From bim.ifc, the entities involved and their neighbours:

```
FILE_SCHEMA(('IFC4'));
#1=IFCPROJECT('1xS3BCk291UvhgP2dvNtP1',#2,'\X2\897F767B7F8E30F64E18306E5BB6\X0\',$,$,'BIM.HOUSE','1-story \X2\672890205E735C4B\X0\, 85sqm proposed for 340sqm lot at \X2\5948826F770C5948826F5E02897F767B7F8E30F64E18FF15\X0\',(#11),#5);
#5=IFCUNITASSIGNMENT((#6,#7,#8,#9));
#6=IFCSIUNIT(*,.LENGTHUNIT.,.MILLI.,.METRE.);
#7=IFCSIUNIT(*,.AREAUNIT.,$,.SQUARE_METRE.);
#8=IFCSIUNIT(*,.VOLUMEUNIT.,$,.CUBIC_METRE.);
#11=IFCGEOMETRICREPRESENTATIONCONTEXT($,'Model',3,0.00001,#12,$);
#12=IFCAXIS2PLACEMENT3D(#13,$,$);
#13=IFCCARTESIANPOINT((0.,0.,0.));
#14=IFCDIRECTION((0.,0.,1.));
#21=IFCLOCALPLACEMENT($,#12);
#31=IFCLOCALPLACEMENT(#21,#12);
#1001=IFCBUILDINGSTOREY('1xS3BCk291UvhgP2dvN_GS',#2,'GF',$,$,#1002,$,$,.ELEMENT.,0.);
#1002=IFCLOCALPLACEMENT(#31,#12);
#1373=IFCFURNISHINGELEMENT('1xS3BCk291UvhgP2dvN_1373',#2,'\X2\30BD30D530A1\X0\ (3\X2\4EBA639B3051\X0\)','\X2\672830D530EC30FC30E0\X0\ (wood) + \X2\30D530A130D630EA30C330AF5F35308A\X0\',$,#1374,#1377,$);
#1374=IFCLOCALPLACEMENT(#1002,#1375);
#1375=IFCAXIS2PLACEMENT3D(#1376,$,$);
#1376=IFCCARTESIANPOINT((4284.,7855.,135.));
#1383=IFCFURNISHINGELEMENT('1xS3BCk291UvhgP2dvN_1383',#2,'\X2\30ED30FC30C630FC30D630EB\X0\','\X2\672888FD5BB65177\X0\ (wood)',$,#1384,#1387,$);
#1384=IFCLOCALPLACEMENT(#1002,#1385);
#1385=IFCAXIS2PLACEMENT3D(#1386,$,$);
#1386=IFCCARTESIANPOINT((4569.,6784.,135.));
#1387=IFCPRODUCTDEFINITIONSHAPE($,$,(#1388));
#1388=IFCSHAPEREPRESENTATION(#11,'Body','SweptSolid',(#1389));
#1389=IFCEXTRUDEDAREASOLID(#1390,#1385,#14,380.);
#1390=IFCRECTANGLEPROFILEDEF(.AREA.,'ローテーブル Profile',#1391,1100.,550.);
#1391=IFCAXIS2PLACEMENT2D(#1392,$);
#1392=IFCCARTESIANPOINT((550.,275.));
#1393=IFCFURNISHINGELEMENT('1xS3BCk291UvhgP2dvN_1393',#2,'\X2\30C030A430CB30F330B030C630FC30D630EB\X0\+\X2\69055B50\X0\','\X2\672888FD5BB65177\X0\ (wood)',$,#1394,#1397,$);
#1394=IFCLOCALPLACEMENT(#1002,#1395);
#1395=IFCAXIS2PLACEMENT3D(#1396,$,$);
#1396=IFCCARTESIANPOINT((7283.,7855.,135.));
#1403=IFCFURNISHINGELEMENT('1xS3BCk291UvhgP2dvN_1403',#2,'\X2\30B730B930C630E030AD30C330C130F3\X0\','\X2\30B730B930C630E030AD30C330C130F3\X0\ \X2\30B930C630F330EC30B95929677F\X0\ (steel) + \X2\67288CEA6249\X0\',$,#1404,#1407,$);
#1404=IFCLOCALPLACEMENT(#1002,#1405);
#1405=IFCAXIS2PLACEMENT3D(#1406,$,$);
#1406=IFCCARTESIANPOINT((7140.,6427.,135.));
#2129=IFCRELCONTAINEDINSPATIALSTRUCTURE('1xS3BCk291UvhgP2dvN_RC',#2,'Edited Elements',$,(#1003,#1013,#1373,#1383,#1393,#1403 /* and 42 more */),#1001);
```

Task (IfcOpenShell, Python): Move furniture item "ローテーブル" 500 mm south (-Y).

```python
import ifcopenshell
import ifcopenshell.api.geometry
import ifcopenshell.util.placement
import ifcopenshell.util.unit

model = ifcopenshell.open("bim.ifc")
unit_scale = ifcopenshell.util.unit.calculate_unit_scale(model)

item = model.by_guid("1xS3BCk291UvhgP2dvN_1383")
matrix = ifcopenshell.util.placement.get_local_placement(item.ObjectPlacement)
matrix[1, 3] -= 0.5 / unit_scale
ifcopenshell.api.geometry.edit_object_placement(model, product=item, matrix=matrix, is_si=False)

print(ifcopenshell.util.placement.get_local_placement(item.ObjectPlacement).round(3) + 0.0)

model.write("bim-out.ifc")
```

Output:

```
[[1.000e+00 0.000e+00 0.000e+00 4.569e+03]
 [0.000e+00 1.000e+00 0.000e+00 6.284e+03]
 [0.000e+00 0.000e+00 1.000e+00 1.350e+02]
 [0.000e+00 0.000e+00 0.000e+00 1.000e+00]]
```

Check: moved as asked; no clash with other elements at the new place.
